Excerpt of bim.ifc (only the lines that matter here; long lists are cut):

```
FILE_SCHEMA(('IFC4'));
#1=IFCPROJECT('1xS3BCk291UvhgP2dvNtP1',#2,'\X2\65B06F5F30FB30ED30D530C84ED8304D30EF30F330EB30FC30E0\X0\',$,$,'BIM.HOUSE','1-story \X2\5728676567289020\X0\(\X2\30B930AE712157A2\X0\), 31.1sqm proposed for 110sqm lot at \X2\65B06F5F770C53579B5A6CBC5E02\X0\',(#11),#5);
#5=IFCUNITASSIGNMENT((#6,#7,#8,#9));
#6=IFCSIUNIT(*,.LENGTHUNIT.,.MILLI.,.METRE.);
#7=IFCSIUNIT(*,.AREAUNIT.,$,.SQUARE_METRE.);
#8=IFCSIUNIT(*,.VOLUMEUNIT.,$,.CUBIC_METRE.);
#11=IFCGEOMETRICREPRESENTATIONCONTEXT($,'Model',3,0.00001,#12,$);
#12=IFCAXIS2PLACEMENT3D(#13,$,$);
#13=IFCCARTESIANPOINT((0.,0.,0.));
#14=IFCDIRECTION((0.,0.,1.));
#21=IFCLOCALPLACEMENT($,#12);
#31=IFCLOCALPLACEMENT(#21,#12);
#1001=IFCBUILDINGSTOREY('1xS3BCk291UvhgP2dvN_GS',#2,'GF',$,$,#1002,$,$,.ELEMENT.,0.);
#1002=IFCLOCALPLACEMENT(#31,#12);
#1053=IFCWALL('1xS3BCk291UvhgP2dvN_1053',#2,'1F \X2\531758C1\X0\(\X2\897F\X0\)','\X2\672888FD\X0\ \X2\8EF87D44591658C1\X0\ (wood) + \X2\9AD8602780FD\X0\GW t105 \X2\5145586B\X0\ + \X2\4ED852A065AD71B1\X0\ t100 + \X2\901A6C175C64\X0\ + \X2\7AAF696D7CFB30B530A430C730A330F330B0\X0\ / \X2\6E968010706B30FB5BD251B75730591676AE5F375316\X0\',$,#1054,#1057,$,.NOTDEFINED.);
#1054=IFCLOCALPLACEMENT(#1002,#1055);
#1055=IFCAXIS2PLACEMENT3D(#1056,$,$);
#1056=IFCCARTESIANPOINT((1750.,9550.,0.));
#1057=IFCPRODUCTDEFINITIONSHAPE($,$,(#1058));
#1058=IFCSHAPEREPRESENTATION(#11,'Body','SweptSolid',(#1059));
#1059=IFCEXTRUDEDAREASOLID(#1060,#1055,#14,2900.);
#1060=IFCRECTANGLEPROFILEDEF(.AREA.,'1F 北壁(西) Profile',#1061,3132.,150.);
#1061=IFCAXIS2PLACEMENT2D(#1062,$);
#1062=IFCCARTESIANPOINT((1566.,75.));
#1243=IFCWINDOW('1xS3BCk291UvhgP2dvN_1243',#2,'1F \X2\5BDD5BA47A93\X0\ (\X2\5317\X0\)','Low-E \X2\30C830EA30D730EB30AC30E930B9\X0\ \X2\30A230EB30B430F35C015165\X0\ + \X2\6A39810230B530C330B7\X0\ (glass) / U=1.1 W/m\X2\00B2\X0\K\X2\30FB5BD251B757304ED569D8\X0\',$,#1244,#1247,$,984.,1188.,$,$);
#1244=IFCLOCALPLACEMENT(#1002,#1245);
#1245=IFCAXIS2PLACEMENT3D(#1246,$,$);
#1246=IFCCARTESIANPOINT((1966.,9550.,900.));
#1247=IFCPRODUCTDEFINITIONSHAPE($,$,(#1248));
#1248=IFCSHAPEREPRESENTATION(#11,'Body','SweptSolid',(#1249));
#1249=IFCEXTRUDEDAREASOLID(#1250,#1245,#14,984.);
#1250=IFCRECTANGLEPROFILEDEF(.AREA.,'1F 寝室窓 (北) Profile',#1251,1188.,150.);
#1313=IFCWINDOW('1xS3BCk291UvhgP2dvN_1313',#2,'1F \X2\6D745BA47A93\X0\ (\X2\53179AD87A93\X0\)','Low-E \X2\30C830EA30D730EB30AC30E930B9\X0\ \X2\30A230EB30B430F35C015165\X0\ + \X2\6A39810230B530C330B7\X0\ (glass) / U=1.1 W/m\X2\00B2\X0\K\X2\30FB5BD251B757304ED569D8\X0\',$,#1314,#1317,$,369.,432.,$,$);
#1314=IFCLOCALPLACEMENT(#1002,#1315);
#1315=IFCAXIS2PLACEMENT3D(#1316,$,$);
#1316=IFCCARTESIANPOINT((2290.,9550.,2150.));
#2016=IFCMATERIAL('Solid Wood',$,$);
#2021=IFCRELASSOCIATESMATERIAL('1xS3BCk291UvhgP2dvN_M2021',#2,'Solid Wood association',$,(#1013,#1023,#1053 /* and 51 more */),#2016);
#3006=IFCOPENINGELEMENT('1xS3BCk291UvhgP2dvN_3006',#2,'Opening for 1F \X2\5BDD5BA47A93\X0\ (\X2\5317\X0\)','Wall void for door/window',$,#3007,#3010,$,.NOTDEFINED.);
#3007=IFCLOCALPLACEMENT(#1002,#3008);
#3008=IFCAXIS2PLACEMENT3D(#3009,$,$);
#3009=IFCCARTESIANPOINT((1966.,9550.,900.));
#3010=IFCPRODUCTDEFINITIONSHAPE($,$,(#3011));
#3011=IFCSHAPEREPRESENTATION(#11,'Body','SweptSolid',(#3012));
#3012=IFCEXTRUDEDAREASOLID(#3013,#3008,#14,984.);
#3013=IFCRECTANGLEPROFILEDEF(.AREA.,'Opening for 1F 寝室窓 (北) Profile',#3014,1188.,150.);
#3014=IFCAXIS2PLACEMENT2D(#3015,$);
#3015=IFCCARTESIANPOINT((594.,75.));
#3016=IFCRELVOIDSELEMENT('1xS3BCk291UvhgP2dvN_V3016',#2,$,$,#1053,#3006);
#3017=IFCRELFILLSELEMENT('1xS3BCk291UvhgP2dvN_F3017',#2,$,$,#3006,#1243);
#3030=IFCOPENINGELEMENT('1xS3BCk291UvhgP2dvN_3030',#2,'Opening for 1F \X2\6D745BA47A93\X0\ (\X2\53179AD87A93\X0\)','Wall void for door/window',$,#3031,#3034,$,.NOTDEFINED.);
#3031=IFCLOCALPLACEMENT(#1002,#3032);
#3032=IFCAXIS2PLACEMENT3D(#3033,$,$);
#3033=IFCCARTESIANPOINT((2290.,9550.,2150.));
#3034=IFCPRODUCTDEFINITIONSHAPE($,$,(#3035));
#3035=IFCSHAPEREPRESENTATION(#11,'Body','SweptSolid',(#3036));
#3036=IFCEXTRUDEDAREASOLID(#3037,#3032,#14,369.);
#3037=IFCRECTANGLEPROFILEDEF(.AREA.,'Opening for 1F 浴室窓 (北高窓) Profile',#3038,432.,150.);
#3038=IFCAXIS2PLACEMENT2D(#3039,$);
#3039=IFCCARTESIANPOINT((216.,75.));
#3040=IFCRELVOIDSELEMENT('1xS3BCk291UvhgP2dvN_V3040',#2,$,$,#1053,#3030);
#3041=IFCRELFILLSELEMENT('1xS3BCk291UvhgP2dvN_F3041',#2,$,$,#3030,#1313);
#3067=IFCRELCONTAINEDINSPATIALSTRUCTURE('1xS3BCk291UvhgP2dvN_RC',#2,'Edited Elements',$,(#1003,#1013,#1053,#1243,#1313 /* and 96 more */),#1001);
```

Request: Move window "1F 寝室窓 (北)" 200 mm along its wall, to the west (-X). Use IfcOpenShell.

```python
import ifcopenshell
import ifcopenshell.api.geometry
import ifcopenshell.util.placement

model = ifcopenshell.open("bim.ifc")

window = model.by_id(1243)
opening = window.FillsVoids[0].RelatingOpeningElement
wall = opening.VoidsElements[0].RelatingBuildingElement

wall_matrix = ifcopenshell.util.placement.get_local_placement(wall.ObjectPlacement)
shift = wall_matrix[:3, 0] * -200.0
before = ifcopenshell.util.placement.get_local_placement(window.ObjectPlacement)[:3, 3].copy()

# The window is not placed relative to its opening, so move both.
for product in (opening, window):
    matrix = ifcopenshell.util.placement.get_local_placement(product.ObjectPlacement)
    matrix[:3, 3] += shift
    ifcopenshell.api.geometry.edit_object_placement(model, product=product, matrix=matrix, is_si=False)

after = ifcopenshell.util.placement.get_local_placement(window.ObjectPlacement)[:3, 3]
print("window moved by", (after - before).round(3) + 0.0)

model.write("bim_rev.ifc")
```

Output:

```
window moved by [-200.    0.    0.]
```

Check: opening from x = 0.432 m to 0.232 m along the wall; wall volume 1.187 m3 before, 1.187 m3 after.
